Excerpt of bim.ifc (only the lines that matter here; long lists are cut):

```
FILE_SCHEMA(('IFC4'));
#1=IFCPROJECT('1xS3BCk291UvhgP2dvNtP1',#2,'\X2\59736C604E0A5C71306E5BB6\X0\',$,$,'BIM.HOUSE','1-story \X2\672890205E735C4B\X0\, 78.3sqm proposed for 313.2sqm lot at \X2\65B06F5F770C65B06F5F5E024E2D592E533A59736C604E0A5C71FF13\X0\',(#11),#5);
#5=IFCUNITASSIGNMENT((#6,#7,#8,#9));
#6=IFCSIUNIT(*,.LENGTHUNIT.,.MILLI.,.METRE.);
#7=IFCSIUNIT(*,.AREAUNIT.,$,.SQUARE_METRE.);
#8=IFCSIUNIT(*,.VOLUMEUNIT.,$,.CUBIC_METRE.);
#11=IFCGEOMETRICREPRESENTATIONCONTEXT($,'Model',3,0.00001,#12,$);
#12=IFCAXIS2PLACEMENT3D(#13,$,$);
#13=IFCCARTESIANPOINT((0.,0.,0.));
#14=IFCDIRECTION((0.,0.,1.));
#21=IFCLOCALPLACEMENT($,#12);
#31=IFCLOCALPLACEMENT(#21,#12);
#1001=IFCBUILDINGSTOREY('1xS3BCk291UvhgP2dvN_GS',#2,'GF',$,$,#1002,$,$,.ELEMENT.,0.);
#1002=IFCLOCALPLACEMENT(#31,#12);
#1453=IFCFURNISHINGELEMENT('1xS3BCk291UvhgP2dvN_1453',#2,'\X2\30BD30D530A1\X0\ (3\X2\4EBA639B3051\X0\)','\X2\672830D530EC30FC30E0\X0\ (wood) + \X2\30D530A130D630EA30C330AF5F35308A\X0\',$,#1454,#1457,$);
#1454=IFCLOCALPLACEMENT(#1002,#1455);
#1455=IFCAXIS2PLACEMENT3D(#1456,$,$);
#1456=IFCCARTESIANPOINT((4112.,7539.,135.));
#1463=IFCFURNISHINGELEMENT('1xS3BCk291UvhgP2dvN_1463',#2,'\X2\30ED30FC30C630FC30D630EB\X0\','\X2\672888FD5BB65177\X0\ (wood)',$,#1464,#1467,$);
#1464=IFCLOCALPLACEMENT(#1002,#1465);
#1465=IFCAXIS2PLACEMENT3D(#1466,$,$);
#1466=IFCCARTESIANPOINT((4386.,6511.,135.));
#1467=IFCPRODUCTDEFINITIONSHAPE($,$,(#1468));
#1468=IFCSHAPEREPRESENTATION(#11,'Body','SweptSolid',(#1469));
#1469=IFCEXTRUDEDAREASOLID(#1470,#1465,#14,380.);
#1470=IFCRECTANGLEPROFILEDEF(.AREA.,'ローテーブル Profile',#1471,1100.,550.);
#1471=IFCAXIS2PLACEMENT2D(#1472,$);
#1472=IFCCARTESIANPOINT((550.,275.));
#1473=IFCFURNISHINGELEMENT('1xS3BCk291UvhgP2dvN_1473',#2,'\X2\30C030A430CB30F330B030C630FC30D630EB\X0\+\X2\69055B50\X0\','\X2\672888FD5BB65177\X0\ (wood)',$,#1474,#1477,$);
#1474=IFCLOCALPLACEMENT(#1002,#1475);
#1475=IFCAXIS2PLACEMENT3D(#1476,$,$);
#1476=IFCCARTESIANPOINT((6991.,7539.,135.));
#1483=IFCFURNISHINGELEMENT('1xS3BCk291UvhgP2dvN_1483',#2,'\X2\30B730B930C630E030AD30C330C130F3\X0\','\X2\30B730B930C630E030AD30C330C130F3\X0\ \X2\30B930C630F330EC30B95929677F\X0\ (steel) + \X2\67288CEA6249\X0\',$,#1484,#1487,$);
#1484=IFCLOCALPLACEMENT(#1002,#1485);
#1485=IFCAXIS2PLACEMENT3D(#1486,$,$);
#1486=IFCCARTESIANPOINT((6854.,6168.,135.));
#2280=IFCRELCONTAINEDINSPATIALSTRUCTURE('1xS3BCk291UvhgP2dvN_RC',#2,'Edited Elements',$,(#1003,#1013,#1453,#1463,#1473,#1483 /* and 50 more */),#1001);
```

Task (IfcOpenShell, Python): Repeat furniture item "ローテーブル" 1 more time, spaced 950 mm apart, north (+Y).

```python
import numpy as np
import ifcopenshell
import ifcopenshell.api.geometry
import ifcopenshell.api.root
import ifcopenshell.util.element
import ifcopenshell.util.placement
import ifcopenshell.util.unit

model = ifcopenshell.open("bim.ifc")
unit_scale = ifcopenshell.util.unit.calculate_unit_scale(model)


def reuse_history(source, copy):
    """copy_class also copies each property set's owner history, people and application; keep the originals."""
    for rel in copy.IsDefinedBy:
        if rel.is_a("IfcRelDefinesByProperties") and (history := rel.RelatingPropertyDefinition.OwnerHistory):
            rel.RelatingPropertyDefinition.OwnerHistory = source.OwnerHistory
            ifcopenshell.util.element.remove_deep2(model, history)


source = model.by_guid("1xS3BCk291UvhgP2dvN_1463")
base = ifcopenshell.util.placement.get_local_placement(source.ObjectPlacement)
step = np.array([0.0, 1.0, 0.0]) * 0.95 / unit_scale

for i in range(1, 2):
    copy = ifcopenshell.api.root.copy_class(model, product=source)
    copy.Representation = ifcopenshell.util.element.copy_deep(
        model, source.Representation, exclude=["IfcGeometricRepresentationContext", "IfcRepresentationMap"]
    )
    reuse_history(source, copy)
    matrix = base.copy()
    matrix[:3, 3] += i * step
    print("added at", matrix[:3, 3].round(3) + 0.0)
    ifcopenshell.api.geometry.edit_object_placement(model, product=copy, matrix=matrix, is_si=False)

model.write("bim-out.ifc")
```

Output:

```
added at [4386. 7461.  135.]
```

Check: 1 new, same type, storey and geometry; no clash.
